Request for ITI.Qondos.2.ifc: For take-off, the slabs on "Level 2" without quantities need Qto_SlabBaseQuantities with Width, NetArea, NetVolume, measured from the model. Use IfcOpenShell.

First a look at what the model holds.

```python
import ifcopenshell
import ifcopenshell.util.element
import ifcopenshell.util.unit

model = ifcopenshell.open("ITI.Qondos.2.ifc")
print(model.schema)
for unit_type in ("LENGTHUNIT", "AREAUNIT", "VOLUMEUNIT"):
    print(unit_type, ifcopenshell.util.unit.calculate_unit_scale(model, unit_type))
storey = next(s for s in model.by_type("IfcBuildingStorey") if s.Name == "Level 2")
slabs = [e for e in ifcopenshell.util.element.get_decomposition(storey) if e.is_a("IfcSlab")]
for e in sorted(slabs, key=lambda e: e.id()):
    print(e.id(), e.is_a(), e.Name, list(ifcopenshell.util.element.get_psets(e, qtos_only=True)), sep=" | ")
```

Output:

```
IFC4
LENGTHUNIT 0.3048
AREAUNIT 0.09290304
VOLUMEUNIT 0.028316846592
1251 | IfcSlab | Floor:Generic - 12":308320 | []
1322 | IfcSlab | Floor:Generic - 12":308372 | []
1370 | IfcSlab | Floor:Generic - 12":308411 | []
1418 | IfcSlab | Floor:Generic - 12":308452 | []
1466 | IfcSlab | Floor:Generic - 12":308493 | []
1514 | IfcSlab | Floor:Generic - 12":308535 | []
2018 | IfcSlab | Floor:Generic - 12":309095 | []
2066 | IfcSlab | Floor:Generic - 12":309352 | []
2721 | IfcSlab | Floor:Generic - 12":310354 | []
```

```python
import ifcopenshell
import ifcopenshell.api.pset
import ifcopenshell.geom
import ifcopenshell.util.element
import ifcopenshell.util.shape
import ifcopenshell.util.unit

model = ifcopenshell.open("ITI.Qondos.2.ifc")
unit_scale = ifcopenshell.util.unit.calculate_unit_scale(model)
area_scale = ifcopenshell.util.unit.calculate_unit_scale(model, "AREAUNIT")
volume_scale = ifcopenshell.util.unit.calculate_unit_scale(model, "VOLUMEUNIT")
settings = ifcopenshell.geom.settings()

storey = next(s for s in model.by_type("IfcBuildingStorey") if s.Name == "Level 2")
slabs = [e for e in ifcopenshell.util.element.get_decomposition(storey) if e.is_a("IfcSlab")]

for e in sorted(slabs, key=lambda e: e.id()):
    if ifcopenshell.util.element.get_psets(e, qtos_only=True, should_inherit=False):
        continue
    # Geometry comes back in metres, in the element's own axes.
    shape = ifcopenshell.geom.create_shape(settings, e)
    values = {
        "Width": ifcopenshell.util.shape.get_z(shape.geometry) / unit_scale,
        "NetArea": ifcopenshell.util.shape.get_footprint_area(shape.geometry) / area_scale,
        "NetVolume": ifcopenshell.util.shape.get_volume(shape.geometry) / volume_scale,
    }
    qto = ifcopenshell.api.pset.add_qto(model, product=e, name="Qto_SlabBaseQuantities")
    ifcopenshell.api.pset.edit_qto(model, qto=qto, properties=values)
    print(e.id(), {k: round(v, 3) for k, v in values.items()})

model.write("ITI.Qondos.2_edited.ifc")
```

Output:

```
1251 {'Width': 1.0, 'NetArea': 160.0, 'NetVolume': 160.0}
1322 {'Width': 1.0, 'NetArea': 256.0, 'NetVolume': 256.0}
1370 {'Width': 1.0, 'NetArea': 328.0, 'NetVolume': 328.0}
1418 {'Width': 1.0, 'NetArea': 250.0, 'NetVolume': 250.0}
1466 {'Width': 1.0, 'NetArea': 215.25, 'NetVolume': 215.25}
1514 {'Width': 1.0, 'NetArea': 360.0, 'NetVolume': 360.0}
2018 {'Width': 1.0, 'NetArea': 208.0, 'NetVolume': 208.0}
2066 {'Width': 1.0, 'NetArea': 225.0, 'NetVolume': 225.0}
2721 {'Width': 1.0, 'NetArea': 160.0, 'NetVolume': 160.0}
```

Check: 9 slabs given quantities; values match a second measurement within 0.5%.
